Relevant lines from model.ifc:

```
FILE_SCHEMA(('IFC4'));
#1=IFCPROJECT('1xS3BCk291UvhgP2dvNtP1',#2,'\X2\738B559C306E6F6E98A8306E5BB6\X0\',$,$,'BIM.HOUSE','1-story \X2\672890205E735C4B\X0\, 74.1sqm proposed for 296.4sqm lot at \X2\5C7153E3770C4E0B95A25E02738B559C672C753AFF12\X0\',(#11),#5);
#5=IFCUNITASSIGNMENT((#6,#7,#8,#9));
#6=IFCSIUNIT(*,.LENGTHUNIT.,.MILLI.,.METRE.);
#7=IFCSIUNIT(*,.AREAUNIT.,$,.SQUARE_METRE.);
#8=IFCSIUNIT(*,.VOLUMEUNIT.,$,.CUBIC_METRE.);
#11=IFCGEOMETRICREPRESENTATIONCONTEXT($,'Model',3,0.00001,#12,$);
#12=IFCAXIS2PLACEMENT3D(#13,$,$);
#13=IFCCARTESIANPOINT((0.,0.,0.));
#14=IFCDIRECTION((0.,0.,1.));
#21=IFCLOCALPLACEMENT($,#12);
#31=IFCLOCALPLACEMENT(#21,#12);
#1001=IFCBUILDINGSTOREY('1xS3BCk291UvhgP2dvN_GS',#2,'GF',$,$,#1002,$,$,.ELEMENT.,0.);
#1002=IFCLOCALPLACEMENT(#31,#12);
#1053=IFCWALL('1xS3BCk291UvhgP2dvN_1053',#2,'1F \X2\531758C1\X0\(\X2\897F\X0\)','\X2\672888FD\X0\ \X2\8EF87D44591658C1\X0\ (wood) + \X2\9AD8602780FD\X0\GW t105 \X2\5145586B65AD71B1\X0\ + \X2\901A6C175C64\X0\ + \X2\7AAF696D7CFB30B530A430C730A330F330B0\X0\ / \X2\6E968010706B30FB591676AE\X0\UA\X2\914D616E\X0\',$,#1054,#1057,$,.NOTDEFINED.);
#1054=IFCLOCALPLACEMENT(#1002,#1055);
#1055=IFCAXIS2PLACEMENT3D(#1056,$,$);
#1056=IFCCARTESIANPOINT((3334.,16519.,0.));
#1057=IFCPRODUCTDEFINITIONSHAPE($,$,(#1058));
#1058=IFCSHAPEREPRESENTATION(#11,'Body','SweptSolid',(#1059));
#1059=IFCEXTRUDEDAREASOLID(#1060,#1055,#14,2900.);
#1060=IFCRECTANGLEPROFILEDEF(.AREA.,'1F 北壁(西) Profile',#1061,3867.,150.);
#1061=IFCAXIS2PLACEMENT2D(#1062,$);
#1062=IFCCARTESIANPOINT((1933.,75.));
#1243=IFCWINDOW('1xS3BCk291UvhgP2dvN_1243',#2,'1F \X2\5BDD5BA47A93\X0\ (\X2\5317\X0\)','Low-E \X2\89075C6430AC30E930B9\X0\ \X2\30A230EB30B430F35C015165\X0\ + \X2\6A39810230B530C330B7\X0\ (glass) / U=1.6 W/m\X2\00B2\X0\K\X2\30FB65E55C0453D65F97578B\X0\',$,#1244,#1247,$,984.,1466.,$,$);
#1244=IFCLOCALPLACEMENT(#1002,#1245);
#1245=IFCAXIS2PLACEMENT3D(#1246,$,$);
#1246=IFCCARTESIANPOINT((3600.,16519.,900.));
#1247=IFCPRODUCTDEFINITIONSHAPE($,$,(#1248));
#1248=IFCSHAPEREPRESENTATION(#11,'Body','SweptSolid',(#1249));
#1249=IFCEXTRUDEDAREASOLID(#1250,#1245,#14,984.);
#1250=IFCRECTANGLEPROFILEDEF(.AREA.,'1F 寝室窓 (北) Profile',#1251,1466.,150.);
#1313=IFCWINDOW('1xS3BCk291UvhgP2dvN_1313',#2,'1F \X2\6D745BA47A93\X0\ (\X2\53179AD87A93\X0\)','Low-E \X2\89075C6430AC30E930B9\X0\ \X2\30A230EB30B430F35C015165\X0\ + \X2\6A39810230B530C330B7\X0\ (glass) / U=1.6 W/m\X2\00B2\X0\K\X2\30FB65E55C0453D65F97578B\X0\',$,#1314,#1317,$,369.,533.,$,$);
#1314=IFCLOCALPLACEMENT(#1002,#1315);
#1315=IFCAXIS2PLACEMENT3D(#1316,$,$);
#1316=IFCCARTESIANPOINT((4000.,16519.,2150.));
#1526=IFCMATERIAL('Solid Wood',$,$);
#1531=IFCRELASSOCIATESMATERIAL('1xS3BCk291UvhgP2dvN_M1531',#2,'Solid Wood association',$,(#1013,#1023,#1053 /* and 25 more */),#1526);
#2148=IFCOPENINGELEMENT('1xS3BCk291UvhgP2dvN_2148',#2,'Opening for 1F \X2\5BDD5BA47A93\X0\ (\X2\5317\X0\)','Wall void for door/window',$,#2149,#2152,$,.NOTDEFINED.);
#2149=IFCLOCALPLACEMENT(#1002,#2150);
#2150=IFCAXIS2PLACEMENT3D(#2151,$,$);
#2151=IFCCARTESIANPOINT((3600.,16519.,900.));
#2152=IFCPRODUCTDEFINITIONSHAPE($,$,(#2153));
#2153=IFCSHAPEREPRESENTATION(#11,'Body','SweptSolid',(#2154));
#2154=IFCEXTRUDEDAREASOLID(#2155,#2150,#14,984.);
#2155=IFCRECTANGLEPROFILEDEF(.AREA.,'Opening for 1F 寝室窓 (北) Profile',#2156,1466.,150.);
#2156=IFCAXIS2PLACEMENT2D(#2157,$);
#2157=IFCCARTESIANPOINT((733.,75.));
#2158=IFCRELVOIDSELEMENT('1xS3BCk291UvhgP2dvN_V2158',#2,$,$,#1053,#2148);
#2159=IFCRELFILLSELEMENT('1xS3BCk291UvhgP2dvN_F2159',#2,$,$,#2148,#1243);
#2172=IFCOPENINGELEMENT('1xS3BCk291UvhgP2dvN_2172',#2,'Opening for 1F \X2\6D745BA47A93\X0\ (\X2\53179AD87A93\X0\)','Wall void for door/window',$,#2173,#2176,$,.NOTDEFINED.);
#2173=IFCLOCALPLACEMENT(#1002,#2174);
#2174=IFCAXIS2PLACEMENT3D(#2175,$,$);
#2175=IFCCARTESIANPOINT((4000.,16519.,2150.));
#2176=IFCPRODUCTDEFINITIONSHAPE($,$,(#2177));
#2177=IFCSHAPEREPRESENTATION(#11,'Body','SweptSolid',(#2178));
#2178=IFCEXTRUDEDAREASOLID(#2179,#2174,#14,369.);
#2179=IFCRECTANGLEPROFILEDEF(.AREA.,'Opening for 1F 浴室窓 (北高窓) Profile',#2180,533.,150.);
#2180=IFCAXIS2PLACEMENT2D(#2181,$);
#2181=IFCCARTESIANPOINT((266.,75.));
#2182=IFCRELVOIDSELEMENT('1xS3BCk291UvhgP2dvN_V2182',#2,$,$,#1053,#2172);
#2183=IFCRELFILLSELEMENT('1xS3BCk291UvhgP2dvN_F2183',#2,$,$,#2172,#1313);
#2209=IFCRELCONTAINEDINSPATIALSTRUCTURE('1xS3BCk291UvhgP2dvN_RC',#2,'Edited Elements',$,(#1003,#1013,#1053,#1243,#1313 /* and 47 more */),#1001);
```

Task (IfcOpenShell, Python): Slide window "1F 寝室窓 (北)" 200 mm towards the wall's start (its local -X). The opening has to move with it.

```python
import ifcopenshell
import ifcopenshell.api.geometry
import ifcopenshell.util.placement
import ifcopenshell.util.unit

model = ifcopenshell.open("model.ifc")
unit_scale = ifcopenshell.util.unit.calculate_unit_scale(model)

window = model.by_id(1243)
opening = window.FillsVoids[0].RelatingOpeningElement
wall = opening.VoidsElements[0].RelatingBuildingElement

wall_matrix = ifcopenshell.util.placement.get_local_placement(wall.ObjectPlacement)
shift = wall_matrix[:3, 0] * -0.2 / unit_scale
before = ifcopenshell.util.placement.get_local_placement(window.ObjectPlacement)[:3, 3].copy()

# The window is not placed relative to its opening, so move both.
for product in (opening, window):
    matrix = ifcopenshell.util.placement.get_local_placement(product.ObjectPlacement)
    matrix[:3, 3] += shift
    ifcopenshell.api.geometry.edit_object_placement(model, product=product, matrix=matrix, is_si=False)

after = ifcopenshell.util.placement.get_local_placement(window.ObjectPlacement)[:3, 3]
print("window moved by", (after - before).round(3) + 0.0)

model.write("model-out.ifc")
```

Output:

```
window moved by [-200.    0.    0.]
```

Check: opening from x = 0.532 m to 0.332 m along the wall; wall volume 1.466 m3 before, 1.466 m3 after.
